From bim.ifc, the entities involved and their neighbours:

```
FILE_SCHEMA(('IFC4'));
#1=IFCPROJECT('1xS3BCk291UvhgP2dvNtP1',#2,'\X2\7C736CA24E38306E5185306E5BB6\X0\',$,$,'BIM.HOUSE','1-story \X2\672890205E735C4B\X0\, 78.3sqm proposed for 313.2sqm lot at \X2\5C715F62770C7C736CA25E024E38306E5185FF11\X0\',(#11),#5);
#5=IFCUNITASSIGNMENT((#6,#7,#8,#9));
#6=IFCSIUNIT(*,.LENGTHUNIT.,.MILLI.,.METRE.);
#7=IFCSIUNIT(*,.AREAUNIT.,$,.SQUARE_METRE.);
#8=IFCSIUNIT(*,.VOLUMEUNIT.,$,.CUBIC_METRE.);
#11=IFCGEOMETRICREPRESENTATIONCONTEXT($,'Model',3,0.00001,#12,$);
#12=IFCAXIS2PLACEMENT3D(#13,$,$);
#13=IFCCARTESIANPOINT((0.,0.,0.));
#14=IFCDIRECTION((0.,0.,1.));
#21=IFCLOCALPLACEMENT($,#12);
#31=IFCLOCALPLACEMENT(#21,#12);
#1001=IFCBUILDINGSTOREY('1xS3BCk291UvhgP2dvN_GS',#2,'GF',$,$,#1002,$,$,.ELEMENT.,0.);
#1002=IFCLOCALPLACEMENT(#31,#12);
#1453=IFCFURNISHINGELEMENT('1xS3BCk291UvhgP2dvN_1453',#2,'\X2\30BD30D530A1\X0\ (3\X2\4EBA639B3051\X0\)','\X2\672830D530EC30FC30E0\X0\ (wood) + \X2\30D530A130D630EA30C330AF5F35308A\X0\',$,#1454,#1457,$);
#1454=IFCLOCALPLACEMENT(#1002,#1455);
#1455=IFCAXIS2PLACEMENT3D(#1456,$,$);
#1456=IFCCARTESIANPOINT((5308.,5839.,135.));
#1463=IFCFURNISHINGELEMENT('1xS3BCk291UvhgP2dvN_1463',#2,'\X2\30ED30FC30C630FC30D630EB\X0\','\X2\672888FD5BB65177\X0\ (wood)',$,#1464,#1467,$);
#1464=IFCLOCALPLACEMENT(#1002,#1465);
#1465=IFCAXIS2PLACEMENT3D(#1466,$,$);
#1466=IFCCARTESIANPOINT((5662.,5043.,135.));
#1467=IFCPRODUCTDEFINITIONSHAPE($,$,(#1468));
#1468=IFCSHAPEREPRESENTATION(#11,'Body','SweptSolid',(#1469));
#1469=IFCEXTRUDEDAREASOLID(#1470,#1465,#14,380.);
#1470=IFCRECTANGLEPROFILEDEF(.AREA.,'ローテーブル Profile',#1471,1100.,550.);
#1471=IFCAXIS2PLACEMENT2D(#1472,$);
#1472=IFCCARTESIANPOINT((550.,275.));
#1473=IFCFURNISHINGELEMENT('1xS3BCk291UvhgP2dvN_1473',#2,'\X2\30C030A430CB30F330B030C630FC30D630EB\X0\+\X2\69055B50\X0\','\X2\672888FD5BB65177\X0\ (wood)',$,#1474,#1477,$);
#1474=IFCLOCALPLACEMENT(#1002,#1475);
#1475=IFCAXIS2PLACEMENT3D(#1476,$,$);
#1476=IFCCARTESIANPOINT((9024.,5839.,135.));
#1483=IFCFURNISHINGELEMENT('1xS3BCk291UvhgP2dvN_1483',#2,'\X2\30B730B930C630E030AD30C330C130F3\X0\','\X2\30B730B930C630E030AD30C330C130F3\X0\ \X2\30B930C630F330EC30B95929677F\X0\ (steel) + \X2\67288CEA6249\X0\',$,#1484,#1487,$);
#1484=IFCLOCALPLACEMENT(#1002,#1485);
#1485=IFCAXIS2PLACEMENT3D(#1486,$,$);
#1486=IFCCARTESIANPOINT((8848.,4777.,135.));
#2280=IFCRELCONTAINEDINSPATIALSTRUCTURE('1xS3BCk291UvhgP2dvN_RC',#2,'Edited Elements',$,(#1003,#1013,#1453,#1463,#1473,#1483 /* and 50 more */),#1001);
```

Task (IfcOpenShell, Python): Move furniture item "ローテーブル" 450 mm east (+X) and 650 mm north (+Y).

```python
import ifcopenshell
import ifcopenshell.api.geometry
import ifcopenshell.util.placement

model = ifcopenshell.open("bim.ifc")

item = model.by_id(1463)
matrix = ifcopenshell.util.placement.get_local_placement(item.ObjectPlacement)
matrix[0, 3] += 450.0
matrix[1, 3] += 650.0
ifcopenshell.api.geometry.edit_object_placement(model, product=item, matrix=matrix, is_si=False)

print(ifcopenshell.util.placement.get_local_placement(item.ObjectPlacement).round(3) + 0.0)

model.write("bim_v2.ifc")
```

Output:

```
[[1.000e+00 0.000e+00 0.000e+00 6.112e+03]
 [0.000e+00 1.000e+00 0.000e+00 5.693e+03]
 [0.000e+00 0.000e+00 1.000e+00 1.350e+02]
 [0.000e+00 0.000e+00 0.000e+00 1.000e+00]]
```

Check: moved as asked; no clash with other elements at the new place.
